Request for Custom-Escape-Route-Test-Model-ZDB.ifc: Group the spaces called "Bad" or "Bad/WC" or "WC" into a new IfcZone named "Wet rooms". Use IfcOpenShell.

First a look at what the model holds.

```python
import ifcopenshell

model = ifcopenshell.open("Custom-Escape-Route-Test-Model-ZDB.ifc")
print(model.schema)
seen = {}
for space in model.by_type("IfcSpace"):
    seen[space.LongName] = seen.get(space.LongName, 0) + 1
for name, count in sorted(seen.items(), key=str):
    print(count, "x", name)
print("zones:", [z.Name for z in model.by_type("IfcZone")][:20])
```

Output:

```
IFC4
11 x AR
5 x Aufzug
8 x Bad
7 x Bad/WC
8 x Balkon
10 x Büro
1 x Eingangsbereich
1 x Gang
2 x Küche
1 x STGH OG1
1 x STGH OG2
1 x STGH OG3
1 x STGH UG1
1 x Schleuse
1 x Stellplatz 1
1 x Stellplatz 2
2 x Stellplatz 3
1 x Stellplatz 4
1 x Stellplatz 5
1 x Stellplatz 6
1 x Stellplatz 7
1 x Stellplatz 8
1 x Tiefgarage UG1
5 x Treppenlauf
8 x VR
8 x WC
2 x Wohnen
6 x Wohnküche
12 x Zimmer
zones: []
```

```python
import ifcopenshell
import ifcopenshell.api.group
import ifcopenshell.api.root

model = ifcopenshell.open("Custom-Escape-Route-Test-Model-ZDB.ifc")

names = {"Bad", "Bad/WC", "WC"}
spaces = [s for s in model.by_type("IfcSpace") if s.LongName in names]

zone = ifcopenshell.api.root.create_entity(model, ifc_class="IfcZone", name="Wet rooms")
ifcopenshell.api.group.assign_group(model, products=spaces, group=zone)
print(len(spaces), "spaces in", zone.Name)

model.write("Custom-Escape-Route-Test-Model-ZDB_updated.ifc")
```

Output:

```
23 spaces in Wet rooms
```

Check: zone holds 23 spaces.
